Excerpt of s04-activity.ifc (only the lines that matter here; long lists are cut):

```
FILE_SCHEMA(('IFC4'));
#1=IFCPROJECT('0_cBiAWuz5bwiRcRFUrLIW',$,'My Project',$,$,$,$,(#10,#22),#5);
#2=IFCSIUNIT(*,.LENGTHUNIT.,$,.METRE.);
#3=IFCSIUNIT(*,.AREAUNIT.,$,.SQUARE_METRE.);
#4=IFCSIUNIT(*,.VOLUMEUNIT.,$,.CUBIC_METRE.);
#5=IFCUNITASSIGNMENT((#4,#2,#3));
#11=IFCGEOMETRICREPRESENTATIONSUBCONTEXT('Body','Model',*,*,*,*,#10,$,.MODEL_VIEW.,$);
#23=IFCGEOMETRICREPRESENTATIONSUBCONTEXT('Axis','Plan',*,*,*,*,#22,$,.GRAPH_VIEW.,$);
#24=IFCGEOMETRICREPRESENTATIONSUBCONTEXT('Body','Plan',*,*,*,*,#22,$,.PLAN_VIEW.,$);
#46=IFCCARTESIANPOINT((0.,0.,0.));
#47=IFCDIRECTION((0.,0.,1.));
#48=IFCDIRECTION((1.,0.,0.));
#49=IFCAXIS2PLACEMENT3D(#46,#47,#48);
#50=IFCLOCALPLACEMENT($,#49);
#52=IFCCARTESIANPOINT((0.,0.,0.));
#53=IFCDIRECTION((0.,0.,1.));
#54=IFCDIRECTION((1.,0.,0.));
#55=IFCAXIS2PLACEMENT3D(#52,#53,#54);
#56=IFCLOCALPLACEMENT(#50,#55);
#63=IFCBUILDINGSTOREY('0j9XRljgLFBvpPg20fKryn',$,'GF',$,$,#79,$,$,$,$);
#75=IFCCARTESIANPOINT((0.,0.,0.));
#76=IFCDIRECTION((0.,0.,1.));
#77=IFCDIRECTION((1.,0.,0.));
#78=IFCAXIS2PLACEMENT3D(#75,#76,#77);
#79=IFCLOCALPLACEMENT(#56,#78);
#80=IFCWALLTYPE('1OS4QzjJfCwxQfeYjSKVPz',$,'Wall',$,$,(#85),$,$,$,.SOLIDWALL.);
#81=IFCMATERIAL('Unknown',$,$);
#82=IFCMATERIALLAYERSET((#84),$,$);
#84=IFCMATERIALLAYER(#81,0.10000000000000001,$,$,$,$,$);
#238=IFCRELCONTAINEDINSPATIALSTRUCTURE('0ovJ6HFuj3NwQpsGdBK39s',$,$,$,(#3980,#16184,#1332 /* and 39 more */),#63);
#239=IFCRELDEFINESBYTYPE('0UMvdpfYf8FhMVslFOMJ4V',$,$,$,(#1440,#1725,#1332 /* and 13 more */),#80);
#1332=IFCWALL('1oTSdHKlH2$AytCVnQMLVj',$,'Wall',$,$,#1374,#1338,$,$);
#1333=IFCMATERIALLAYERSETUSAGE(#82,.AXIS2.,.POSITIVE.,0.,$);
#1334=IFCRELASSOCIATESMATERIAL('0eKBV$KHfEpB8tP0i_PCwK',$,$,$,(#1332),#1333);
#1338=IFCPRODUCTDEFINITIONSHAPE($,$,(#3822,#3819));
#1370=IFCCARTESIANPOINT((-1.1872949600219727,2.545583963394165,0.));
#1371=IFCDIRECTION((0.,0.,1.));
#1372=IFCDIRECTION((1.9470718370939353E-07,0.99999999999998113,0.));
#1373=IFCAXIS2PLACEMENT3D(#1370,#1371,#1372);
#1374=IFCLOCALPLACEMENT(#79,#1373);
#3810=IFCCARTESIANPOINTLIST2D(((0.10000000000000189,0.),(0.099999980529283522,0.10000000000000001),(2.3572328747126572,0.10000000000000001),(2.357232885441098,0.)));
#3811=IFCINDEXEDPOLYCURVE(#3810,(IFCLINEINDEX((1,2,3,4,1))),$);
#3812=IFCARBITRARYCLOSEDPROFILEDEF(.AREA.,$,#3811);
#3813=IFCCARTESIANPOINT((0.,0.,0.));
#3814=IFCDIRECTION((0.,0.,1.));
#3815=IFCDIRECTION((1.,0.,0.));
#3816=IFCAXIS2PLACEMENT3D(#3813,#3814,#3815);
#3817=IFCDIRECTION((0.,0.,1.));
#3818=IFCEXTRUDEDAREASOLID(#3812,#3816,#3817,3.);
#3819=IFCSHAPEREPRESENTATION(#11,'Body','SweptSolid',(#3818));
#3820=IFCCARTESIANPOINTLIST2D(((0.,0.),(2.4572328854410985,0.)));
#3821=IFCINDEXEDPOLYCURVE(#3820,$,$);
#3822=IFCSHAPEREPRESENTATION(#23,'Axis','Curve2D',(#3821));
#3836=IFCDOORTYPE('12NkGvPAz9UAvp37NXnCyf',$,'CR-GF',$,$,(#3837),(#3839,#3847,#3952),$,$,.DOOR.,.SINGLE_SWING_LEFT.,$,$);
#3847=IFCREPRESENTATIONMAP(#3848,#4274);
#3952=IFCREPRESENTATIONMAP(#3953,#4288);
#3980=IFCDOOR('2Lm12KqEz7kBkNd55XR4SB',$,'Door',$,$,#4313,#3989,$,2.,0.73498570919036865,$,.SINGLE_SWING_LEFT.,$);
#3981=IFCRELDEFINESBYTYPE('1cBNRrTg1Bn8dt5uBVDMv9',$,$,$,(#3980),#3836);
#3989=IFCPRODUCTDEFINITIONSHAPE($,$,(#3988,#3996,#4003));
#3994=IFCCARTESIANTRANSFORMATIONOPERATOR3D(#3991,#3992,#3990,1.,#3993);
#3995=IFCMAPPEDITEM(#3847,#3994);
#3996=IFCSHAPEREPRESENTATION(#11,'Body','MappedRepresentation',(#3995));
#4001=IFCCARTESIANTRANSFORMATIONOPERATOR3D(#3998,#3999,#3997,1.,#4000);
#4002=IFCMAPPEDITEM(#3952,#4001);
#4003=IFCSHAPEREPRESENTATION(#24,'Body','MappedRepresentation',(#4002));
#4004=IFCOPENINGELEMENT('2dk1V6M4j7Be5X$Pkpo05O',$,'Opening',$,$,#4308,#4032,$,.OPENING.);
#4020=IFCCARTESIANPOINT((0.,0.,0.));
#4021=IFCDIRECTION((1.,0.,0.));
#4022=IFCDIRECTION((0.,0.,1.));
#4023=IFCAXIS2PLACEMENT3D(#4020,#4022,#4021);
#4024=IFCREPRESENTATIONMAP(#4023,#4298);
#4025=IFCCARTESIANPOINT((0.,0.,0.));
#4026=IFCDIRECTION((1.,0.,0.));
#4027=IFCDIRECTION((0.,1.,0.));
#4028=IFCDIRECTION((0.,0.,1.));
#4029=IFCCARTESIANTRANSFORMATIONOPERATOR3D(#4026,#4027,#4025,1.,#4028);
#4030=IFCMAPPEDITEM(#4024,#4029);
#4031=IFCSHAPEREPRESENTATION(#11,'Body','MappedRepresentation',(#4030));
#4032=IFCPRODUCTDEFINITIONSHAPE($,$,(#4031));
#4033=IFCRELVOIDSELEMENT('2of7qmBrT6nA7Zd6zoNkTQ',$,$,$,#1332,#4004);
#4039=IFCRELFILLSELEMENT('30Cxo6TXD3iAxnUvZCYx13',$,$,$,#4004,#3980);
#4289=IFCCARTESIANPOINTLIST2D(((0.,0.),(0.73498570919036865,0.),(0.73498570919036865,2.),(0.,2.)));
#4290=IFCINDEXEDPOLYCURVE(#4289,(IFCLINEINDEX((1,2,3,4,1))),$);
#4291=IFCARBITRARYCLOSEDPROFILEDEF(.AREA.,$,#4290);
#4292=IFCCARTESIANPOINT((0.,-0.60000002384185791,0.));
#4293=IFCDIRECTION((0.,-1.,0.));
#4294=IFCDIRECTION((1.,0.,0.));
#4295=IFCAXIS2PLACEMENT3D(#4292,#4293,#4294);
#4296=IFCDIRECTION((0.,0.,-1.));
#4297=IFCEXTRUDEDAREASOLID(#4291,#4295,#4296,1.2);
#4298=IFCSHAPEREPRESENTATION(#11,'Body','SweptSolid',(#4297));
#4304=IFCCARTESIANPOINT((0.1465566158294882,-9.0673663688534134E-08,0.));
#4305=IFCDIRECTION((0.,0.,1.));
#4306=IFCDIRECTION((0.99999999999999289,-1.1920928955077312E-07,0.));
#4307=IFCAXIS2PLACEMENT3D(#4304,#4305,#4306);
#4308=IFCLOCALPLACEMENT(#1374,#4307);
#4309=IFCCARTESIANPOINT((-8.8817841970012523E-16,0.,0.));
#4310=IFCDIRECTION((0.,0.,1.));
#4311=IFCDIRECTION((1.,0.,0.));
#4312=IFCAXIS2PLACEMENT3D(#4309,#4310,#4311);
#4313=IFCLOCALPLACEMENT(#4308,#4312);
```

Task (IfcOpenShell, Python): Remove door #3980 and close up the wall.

```python
import ifcopenshell
import ifcopenshell.api.feature
import ifcopenshell.api.root
import ifcopenshell.geom
import ifcopenshell.util.shape

model = ifcopenshell.open("s04-activity.ifc")
settings = ifcopenshell.geom.settings()


def volume(element):
    """Net volume in cubic metres, openings subtracted."""
    shape = ifcopenshell.geom.create_shape(settings, element)
    return ifcopenshell.util.shape.get_volume(shape.geometry)


door = model.by_guid("2Lm12KqEz7kBkNd55XR4SB")
opening = door.FillsVoids[0].RelatingOpeningElement
wall = opening.VoidsElements[0].RelatingBuildingElement
before = volume(wall)

ifcopenshell.api.root.remove_product(model, product=door)
ifcopenshell.api.feature.remove_feature(model, feature=opening)

after = volume(wall)

print(f"wall volume {before:.3f} -> {after:.3f} m3")

model.write("s04-activity_edited.ifc")
```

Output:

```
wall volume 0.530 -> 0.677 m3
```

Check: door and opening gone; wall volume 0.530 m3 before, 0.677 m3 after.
